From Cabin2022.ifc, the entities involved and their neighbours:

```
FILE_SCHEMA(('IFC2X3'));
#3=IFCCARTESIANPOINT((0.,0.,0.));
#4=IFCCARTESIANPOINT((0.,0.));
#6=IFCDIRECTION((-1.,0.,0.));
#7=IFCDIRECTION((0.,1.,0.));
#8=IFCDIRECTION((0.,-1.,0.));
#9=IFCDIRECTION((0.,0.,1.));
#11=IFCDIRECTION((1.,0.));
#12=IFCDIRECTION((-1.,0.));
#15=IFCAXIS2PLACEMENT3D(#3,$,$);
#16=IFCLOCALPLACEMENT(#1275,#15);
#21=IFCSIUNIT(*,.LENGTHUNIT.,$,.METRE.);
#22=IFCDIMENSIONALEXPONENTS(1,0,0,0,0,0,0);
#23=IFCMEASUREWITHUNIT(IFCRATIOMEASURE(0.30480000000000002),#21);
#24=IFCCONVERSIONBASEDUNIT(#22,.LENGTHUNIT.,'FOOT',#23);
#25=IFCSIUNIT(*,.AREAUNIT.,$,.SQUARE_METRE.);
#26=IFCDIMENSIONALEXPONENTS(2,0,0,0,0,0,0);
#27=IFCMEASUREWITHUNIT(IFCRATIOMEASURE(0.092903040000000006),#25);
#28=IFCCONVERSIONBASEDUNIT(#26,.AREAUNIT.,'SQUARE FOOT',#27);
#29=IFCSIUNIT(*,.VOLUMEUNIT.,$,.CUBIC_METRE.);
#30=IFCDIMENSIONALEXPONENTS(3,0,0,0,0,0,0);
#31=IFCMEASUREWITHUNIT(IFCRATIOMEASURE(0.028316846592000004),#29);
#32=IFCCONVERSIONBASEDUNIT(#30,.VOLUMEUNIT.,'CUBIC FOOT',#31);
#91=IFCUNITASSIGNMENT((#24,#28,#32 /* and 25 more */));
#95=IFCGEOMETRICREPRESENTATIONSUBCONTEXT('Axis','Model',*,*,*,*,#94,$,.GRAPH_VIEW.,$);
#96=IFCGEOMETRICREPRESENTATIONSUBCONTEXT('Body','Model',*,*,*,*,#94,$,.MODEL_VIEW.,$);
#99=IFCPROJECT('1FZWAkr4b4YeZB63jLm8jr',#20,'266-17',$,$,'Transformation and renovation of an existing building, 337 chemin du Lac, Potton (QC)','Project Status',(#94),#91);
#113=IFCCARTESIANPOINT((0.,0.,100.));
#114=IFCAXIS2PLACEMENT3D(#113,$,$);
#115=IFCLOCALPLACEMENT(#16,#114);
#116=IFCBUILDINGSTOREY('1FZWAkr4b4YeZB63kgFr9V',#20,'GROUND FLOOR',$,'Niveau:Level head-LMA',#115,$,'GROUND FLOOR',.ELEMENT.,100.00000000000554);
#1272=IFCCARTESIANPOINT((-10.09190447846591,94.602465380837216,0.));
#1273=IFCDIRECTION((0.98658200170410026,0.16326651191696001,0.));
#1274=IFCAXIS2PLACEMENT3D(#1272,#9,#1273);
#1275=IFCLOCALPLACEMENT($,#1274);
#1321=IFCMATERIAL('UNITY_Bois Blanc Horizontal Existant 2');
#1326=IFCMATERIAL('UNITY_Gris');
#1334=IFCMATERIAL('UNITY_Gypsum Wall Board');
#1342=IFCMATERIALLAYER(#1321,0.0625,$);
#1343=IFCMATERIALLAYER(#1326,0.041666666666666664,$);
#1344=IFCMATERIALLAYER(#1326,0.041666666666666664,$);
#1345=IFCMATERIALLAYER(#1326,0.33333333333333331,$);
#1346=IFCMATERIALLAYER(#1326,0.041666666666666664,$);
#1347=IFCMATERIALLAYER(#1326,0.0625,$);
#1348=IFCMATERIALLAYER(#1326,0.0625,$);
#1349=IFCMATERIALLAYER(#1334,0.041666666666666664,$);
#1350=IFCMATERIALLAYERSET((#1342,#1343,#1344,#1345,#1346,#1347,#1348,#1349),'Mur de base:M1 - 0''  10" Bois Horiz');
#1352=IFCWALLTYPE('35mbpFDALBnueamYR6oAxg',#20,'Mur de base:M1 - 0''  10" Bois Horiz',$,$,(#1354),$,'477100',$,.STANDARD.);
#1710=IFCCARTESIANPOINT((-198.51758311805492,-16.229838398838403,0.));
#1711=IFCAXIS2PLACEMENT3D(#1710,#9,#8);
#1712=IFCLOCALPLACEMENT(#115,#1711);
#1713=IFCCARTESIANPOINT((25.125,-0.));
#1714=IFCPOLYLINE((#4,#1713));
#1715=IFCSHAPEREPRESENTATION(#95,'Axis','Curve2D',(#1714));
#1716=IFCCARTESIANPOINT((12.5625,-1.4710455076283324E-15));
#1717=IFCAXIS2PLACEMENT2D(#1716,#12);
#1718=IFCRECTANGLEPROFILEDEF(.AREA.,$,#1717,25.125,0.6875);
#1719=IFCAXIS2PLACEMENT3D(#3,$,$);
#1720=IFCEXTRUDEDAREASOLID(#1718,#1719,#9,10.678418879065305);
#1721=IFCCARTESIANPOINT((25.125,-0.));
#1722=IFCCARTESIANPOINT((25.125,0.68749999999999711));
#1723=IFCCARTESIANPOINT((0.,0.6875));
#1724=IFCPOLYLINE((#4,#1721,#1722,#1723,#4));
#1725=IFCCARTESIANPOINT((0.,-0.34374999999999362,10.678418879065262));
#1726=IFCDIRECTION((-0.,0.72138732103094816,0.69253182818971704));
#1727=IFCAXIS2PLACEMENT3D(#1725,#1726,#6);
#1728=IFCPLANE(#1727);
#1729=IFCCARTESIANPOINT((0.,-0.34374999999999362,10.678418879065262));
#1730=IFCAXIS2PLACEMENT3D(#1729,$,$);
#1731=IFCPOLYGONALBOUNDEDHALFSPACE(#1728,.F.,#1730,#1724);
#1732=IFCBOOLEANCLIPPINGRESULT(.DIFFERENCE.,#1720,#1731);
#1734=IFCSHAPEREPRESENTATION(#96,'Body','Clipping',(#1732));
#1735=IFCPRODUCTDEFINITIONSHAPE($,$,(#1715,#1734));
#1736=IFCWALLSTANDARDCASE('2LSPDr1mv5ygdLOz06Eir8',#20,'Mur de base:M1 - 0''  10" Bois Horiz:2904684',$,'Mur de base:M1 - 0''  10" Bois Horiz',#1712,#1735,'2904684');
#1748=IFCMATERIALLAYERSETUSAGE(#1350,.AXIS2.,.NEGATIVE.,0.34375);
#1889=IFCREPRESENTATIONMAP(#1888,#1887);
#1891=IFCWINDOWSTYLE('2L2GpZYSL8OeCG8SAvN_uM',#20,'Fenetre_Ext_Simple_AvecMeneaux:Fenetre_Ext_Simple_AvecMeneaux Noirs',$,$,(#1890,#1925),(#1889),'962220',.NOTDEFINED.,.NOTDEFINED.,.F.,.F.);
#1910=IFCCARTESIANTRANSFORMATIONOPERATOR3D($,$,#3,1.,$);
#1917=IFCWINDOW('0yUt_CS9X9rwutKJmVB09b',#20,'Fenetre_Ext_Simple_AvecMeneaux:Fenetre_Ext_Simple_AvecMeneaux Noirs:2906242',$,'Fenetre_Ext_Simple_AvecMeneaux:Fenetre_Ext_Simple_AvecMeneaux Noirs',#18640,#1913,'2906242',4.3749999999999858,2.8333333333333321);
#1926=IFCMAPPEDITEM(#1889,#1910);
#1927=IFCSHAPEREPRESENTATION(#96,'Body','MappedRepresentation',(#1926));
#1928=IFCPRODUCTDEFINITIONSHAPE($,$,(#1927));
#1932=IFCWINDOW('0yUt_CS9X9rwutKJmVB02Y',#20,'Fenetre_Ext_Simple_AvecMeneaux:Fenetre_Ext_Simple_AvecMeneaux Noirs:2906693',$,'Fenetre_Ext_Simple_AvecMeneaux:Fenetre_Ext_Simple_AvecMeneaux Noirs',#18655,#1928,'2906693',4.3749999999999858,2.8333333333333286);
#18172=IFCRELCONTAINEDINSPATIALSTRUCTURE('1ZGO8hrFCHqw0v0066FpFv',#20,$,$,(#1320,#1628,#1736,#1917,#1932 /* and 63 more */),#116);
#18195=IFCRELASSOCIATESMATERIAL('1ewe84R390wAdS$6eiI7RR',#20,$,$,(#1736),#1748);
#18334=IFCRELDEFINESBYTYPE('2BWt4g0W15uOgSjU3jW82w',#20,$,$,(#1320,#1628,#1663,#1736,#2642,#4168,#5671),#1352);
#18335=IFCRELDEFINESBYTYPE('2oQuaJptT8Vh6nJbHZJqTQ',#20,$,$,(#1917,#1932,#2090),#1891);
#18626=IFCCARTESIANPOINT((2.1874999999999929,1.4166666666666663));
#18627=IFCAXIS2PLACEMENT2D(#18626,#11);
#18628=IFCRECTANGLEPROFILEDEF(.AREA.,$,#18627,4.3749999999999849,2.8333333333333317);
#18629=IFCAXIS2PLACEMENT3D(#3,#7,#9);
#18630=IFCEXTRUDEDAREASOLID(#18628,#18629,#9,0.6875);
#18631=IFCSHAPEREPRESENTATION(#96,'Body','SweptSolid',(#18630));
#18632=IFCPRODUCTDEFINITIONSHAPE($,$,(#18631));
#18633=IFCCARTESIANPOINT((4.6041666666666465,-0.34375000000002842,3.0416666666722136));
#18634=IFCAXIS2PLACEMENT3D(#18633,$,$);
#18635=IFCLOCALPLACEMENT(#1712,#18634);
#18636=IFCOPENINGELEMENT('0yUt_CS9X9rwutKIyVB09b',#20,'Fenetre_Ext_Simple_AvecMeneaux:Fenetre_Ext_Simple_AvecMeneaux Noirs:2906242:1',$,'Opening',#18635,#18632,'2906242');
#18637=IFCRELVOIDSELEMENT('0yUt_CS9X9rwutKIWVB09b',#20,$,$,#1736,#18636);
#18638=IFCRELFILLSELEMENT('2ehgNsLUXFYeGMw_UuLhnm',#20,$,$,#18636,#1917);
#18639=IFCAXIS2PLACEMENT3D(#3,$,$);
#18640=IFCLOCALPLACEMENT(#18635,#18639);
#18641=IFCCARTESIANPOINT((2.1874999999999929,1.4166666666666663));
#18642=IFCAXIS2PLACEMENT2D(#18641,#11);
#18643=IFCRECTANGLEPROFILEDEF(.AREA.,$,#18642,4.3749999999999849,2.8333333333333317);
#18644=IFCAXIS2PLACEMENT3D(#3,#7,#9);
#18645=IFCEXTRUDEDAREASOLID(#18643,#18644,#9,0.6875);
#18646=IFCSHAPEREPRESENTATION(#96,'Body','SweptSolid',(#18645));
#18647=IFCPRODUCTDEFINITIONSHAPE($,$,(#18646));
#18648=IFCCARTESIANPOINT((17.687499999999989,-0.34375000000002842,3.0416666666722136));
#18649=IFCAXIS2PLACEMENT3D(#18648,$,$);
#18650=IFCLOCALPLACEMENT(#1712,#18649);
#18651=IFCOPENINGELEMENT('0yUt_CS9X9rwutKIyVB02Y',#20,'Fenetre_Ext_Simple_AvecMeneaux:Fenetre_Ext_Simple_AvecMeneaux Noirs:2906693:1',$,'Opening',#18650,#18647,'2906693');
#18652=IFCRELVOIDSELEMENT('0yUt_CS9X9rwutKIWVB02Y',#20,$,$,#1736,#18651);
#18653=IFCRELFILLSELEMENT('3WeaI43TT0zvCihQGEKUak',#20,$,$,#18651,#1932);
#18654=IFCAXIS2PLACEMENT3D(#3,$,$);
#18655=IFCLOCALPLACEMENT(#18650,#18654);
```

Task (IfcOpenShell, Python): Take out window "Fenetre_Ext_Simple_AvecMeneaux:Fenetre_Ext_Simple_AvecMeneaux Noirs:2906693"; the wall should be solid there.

```python
import ifcopenshell
import ifcopenshell.api.feature
import ifcopenshell.api.root
import ifcopenshell.geom
import ifcopenshell.util.shape

model = ifcopenshell.open("Cabin2022.ifc")
settings = ifcopenshell.geom.settings()


def volume(element):
    """Net volume in cubic metres, openings subtracted."""
    shape = ifcopenshell.geom.create_shape(settings, element)
    return ifcopenshell.util.shape.get_volume(shape.geometry)


window = model.by_guid("0yUt_CS9X9rwutKJmVB02Y")
opening = window.FillsVoids[0].RelatingOpeningElement
wall = opening.VoidsElements[0].RelatingBuildingElement
before = volume(wall)

ifcopenshell.api.root.remove_product(model, product=window)
ifcopenshell.api.feature.remove_feature(model, feature=opening)

after = volume(wall)

print(f"wall volume {before:.3f} -> {after:.3f} m3")

model.write("Cabin2022_edited.ifc")
```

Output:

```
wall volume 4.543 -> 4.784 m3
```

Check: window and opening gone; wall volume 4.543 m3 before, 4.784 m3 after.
